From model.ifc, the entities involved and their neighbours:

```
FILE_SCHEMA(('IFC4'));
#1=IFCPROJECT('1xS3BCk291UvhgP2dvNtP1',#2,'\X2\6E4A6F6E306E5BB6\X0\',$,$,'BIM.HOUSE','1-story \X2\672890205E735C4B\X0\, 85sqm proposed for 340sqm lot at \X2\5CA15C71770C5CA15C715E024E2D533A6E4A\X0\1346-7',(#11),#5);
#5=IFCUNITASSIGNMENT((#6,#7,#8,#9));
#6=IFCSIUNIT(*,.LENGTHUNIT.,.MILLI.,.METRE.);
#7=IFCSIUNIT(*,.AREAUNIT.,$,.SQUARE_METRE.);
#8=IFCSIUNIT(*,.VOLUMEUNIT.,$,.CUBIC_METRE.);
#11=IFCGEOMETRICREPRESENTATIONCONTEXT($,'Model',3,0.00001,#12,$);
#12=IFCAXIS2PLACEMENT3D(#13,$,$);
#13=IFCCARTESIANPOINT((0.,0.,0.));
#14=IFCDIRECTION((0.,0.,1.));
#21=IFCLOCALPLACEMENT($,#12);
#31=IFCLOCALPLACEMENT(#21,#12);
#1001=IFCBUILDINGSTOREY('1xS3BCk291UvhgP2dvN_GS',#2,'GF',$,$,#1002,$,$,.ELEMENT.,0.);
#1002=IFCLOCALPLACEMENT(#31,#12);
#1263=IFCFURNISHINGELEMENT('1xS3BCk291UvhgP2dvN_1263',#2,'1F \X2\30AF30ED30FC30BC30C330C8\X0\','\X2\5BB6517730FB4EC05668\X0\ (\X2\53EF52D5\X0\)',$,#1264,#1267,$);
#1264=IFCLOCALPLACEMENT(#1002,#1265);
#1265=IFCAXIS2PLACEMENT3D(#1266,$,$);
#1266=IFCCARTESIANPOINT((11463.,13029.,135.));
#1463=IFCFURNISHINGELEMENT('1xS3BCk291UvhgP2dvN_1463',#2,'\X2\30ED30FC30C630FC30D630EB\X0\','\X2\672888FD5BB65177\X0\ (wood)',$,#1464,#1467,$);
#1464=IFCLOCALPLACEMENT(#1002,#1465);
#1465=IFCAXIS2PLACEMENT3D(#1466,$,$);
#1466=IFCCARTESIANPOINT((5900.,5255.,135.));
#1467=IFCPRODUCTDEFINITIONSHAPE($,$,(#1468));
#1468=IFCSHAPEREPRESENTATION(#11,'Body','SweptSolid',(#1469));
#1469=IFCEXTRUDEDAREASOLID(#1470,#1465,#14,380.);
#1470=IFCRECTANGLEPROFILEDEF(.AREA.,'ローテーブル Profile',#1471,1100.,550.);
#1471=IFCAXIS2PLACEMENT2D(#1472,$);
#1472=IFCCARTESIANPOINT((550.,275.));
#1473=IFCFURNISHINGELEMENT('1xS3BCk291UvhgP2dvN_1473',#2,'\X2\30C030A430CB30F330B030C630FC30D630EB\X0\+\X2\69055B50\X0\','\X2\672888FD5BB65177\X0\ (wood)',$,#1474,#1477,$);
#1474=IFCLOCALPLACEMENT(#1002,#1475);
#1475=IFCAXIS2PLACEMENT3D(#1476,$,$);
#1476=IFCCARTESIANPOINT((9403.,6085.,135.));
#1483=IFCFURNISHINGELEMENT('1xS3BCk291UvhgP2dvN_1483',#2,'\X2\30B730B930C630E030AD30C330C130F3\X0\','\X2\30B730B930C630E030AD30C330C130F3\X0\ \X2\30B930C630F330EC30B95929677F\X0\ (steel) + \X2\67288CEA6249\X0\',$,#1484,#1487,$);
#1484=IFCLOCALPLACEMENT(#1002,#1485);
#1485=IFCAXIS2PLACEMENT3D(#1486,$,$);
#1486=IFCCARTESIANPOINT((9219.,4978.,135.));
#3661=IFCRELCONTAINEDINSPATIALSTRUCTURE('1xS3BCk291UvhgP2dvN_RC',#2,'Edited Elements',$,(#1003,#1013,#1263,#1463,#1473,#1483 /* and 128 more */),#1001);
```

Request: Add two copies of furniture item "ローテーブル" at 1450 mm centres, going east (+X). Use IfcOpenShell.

```python
import numpy as np
import ifcopenshell
import ifcopenshell.api.geometry
import ifcopenshell.api.root
import ifcopenshell.util.element
import ifcopenshell.util.placement
import ifcopenshell.util.unit

model = ifcopenshell.open("model.ifc")
unit_scale = ifcopenshell.util.unit.calculate_unit_scale(model)


def reuse_history(source, copy):
    """copy_class also copies each property set's owner history, people and application; keep the originals."""
    for rel in copy.IsDefinedBy:
        if rel.is_a("IfcRelDefinesByProperties") and (history := rel.RelatingPropertyDefinition.OwnerHistory):
            rel.RelatingPropertyDefinition.OwnerHistory = source.OwnerHistory
            ifcopenshell.util.element.remove_deep2(model, history)


source = model.by_guid("1xS3BCk291UvhgP2dvN_1463")
base = ifcopenshell.util.placement.get_local_placement(source.ObjectPlacement)
step = np.array([1.0, 0.0, 0.0]) * 1.45 / unit_scale

for i in range(1, 3):
    copy = ifcopenshell.api.root.copy_class(model, product=source)
    copy.Representation = ifcopenshell.util.element.copy_deep(
        model, source.Representation, exclude=["IfcGeometricRepresentationContext", "IfcRepresentationMap"]
    )
    reuse_history(source, copy)
    matrix = base.copy()
    matrix[:3, 3] += i * step
    print("added at", matrix[:3, 3].round(3) + 0.0)
    ifcopenshell.api.geometry.edit_object_placement(model, product=copy, matrix=matrix, is_si=False)

model.write("model-out.ifc")
```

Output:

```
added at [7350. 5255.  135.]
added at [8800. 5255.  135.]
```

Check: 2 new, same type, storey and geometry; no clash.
